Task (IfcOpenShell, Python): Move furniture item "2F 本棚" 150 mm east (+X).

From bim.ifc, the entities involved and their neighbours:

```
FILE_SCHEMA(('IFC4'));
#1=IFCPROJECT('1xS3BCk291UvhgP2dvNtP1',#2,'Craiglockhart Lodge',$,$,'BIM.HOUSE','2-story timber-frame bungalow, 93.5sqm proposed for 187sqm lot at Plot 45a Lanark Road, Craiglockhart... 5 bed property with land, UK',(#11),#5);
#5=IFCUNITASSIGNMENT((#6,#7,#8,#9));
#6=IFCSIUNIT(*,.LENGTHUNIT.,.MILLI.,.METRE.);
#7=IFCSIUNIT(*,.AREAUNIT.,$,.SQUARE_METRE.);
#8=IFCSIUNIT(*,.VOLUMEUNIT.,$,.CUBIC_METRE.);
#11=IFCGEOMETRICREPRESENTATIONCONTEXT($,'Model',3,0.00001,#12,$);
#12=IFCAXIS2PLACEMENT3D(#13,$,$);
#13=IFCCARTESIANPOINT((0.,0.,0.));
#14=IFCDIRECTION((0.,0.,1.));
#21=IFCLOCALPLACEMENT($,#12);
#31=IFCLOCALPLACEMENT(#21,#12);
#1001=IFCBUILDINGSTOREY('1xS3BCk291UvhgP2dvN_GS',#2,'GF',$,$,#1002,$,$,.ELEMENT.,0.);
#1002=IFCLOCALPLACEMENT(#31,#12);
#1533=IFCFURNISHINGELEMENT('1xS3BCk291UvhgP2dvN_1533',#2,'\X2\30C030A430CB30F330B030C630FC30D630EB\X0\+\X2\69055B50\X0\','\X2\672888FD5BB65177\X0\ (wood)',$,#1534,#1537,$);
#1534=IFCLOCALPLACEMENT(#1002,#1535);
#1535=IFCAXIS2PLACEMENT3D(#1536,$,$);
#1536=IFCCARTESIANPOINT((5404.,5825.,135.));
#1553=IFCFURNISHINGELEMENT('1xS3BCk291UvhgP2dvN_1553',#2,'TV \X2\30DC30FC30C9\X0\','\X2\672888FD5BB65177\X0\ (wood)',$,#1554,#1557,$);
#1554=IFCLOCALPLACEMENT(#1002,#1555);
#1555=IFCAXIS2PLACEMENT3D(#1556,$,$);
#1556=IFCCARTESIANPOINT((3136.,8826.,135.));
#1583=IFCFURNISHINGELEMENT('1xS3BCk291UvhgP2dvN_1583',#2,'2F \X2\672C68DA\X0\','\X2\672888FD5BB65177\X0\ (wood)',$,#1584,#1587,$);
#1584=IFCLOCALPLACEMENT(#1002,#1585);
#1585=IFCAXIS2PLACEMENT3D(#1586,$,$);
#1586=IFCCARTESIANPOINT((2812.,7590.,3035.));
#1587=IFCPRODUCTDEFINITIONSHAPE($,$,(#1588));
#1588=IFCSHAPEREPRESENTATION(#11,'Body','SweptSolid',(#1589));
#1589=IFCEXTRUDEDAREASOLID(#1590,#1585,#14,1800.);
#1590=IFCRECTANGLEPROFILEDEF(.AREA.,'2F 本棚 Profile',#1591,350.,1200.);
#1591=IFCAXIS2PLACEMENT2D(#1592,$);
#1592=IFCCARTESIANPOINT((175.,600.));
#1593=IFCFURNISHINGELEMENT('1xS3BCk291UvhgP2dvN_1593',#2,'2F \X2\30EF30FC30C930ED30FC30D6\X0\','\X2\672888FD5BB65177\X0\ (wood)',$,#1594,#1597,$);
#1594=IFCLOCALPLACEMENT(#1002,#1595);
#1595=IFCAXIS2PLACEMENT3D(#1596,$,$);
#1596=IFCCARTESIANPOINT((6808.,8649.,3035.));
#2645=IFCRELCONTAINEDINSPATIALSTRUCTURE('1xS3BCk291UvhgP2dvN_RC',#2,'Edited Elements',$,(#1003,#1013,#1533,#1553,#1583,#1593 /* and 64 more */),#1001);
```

```python
import ifcopenshell
import ifcopenshell.api.geometry
import ifcopenshell.util.placement
import ifcopenshell.util.unit

model = ifcopenshell.open("bim.ifc")
unit_scale = ifcopenshell.util.unit.calculate_unit_scale(model)

item = model.by_guid("1xS3BCk291UvhgP2dvN_1583")
matrix = ifcopenshell.util.placement.get_local_placement(item.ObjectPlacement)
matrix[0, 3] += 0.15 / unit_scale
ifcopenshell.api.geometry.edit_object_placement(model, product=item, matrix=matrix, is_si=False)

print(ifcopenshell.util.placement.get_local_placement(item.ObjectPlacement).round(3) + 0.0)

model.write("bim-out.ifc")
```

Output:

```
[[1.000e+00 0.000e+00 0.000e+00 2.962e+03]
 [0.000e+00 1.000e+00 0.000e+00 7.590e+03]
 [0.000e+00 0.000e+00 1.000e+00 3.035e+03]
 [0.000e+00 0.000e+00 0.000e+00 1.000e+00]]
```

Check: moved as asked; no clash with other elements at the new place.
